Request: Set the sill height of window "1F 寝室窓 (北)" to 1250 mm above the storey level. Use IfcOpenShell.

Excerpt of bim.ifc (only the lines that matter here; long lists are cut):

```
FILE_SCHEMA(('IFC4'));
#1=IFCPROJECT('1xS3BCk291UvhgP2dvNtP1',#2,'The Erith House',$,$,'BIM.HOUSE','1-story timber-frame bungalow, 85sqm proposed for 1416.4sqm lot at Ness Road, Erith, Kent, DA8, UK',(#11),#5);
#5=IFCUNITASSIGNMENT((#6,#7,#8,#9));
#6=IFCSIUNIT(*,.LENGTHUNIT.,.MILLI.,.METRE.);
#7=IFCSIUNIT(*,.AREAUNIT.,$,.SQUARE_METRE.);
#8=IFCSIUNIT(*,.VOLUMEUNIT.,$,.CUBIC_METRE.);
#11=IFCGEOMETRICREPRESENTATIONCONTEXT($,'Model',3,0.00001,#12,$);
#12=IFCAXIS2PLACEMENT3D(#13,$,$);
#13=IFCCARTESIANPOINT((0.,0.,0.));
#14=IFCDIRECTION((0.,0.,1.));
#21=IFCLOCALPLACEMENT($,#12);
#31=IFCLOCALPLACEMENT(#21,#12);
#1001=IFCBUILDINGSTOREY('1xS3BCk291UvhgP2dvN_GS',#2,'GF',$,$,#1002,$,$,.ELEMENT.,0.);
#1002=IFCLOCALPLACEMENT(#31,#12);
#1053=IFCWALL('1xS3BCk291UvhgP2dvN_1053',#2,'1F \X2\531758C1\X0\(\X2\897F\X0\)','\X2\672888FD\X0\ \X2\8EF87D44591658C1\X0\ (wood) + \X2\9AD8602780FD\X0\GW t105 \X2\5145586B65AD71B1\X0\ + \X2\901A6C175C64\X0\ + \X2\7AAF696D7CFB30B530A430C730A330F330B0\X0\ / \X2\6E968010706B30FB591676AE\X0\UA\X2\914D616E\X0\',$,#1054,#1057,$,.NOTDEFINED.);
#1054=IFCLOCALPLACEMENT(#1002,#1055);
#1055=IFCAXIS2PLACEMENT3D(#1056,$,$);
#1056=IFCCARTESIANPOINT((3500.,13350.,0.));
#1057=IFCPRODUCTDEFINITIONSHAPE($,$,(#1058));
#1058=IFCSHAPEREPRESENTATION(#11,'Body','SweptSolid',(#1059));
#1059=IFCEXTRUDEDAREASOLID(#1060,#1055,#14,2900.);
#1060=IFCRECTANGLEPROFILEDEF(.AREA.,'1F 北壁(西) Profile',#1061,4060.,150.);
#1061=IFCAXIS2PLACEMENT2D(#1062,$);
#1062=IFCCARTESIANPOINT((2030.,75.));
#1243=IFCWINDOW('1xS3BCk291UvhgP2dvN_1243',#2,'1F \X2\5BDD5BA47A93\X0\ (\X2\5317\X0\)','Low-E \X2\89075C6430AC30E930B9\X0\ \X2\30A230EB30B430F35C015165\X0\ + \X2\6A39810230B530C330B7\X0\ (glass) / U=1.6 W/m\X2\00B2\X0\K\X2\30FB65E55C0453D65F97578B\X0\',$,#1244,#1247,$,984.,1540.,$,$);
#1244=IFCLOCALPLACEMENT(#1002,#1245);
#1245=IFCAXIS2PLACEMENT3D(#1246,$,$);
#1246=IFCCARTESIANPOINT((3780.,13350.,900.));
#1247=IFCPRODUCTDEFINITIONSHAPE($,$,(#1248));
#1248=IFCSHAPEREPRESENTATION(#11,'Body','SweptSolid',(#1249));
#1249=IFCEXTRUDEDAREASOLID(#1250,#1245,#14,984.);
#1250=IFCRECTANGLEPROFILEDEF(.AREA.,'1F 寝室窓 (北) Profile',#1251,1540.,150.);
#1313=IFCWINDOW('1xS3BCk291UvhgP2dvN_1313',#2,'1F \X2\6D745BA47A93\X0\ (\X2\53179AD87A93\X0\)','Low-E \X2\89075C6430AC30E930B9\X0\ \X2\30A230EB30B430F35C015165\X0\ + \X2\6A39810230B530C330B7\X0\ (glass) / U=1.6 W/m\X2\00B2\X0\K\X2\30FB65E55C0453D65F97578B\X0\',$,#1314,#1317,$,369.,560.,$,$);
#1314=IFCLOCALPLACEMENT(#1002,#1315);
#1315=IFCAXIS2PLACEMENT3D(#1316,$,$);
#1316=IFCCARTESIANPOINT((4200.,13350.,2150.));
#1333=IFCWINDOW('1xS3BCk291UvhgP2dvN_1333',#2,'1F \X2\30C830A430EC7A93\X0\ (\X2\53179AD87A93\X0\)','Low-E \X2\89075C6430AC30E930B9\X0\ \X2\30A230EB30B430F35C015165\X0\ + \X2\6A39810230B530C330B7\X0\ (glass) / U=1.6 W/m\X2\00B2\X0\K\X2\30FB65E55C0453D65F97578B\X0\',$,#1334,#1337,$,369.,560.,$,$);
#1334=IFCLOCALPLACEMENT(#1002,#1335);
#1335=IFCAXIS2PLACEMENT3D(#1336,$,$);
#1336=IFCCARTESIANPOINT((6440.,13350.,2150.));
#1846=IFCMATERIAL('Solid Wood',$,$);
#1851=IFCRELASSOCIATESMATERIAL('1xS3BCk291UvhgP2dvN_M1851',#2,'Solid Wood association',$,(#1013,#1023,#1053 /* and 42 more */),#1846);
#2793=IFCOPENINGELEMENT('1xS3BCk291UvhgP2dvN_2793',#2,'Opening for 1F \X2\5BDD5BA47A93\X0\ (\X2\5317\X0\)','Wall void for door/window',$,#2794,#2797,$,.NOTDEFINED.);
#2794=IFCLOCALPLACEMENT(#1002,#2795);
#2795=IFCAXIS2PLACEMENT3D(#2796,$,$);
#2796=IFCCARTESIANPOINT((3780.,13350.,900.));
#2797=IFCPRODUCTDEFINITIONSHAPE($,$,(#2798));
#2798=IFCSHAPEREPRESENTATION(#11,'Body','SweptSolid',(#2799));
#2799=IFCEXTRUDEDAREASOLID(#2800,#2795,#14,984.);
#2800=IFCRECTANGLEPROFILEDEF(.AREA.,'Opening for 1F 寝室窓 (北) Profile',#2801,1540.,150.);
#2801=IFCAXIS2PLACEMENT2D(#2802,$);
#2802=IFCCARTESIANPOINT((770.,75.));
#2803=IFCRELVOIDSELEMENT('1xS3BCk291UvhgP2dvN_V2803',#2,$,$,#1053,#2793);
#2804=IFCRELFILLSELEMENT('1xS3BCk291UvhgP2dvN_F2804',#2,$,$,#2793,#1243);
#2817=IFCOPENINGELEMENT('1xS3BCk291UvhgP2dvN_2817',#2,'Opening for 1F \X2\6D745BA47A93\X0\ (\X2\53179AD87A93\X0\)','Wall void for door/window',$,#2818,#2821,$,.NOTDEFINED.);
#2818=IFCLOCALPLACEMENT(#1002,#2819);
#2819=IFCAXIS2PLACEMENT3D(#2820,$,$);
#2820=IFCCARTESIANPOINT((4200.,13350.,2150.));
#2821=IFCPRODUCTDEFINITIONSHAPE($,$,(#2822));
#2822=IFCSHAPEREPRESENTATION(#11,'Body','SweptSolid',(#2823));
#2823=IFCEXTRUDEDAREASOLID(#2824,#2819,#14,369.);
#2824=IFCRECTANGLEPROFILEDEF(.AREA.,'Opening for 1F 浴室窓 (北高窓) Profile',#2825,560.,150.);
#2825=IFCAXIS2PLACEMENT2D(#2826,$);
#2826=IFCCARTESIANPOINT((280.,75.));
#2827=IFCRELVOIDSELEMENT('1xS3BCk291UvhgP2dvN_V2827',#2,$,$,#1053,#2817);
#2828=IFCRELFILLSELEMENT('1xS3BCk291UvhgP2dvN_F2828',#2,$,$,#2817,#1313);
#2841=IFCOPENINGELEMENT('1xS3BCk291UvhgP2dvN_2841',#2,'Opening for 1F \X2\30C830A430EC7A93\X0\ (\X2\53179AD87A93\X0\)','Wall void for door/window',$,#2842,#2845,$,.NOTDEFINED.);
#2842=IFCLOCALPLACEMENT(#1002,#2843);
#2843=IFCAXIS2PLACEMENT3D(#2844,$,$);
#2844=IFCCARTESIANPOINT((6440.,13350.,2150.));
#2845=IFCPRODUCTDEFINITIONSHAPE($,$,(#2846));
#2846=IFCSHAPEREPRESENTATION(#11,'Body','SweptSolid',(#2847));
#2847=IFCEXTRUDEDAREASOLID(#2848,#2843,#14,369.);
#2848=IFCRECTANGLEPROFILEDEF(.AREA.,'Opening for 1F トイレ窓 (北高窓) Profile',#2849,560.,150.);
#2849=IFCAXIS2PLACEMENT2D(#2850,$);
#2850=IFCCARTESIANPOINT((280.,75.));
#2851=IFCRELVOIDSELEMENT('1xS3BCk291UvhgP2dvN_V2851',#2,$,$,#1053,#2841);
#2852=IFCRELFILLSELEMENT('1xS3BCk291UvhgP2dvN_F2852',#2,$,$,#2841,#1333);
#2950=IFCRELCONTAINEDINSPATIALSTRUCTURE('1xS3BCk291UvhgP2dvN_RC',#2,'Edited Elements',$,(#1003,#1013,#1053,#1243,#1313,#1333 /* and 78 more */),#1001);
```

```python
import numpy as np
import ifcopenshell
import ifcopenshell.api.geometry
import ifcopenshell.geom
import ifcopenshell.util.element
import ifcopenshell.util.placement
import ifcopenshell.util.shape
import ifcopenshell.util.unit

model = ifcopenshell.open("bim.ifc")
unit_scale = ifcopenshell.util.unit.calculate_unit_scale(model)

window = model.by_guid("1xS3BCk291UvhgP2dvN_1243")
opening = window.FillsVoids[0].RelatingOpeningElement
storey = ifcopenshell.util.element.get_container(window, ifc_class="IfcBuildingStorey")
level = ifcopenshell.util.placement.get_local_placement(storey.ObjectPlacement)[2, 3]

# The opening's origin need not be at the sill, so measure its lowest point.
shape = ifcopenshell.geom.create_shape(ifcopenshell.geom.settings(), opening)
bottom = ifcopenshell.util.shape.get_shape_bottom_elevation(shape, shape.geometry) / unit_scale
dz = level + 1.25 / unit_scale - bottom

shift = np.array([0.0, 0.0, dz])
# The window is not placed relative to its opening, so move both.
for product in (opening, window):
    matrix = ifcopenshell.util.placement.get_local_placement(product.ObjectPlacement)
    matrix[:3, 3] += shift
    ifcopenshell.api.geometry.edit_object_placement(model, product=product, matrix=matrix, is_si=False)

print(f"moved by {dz * unit_scale:+.3f} m")

model.write("bim-out.ifc")
```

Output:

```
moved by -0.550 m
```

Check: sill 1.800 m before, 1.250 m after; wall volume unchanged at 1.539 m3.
